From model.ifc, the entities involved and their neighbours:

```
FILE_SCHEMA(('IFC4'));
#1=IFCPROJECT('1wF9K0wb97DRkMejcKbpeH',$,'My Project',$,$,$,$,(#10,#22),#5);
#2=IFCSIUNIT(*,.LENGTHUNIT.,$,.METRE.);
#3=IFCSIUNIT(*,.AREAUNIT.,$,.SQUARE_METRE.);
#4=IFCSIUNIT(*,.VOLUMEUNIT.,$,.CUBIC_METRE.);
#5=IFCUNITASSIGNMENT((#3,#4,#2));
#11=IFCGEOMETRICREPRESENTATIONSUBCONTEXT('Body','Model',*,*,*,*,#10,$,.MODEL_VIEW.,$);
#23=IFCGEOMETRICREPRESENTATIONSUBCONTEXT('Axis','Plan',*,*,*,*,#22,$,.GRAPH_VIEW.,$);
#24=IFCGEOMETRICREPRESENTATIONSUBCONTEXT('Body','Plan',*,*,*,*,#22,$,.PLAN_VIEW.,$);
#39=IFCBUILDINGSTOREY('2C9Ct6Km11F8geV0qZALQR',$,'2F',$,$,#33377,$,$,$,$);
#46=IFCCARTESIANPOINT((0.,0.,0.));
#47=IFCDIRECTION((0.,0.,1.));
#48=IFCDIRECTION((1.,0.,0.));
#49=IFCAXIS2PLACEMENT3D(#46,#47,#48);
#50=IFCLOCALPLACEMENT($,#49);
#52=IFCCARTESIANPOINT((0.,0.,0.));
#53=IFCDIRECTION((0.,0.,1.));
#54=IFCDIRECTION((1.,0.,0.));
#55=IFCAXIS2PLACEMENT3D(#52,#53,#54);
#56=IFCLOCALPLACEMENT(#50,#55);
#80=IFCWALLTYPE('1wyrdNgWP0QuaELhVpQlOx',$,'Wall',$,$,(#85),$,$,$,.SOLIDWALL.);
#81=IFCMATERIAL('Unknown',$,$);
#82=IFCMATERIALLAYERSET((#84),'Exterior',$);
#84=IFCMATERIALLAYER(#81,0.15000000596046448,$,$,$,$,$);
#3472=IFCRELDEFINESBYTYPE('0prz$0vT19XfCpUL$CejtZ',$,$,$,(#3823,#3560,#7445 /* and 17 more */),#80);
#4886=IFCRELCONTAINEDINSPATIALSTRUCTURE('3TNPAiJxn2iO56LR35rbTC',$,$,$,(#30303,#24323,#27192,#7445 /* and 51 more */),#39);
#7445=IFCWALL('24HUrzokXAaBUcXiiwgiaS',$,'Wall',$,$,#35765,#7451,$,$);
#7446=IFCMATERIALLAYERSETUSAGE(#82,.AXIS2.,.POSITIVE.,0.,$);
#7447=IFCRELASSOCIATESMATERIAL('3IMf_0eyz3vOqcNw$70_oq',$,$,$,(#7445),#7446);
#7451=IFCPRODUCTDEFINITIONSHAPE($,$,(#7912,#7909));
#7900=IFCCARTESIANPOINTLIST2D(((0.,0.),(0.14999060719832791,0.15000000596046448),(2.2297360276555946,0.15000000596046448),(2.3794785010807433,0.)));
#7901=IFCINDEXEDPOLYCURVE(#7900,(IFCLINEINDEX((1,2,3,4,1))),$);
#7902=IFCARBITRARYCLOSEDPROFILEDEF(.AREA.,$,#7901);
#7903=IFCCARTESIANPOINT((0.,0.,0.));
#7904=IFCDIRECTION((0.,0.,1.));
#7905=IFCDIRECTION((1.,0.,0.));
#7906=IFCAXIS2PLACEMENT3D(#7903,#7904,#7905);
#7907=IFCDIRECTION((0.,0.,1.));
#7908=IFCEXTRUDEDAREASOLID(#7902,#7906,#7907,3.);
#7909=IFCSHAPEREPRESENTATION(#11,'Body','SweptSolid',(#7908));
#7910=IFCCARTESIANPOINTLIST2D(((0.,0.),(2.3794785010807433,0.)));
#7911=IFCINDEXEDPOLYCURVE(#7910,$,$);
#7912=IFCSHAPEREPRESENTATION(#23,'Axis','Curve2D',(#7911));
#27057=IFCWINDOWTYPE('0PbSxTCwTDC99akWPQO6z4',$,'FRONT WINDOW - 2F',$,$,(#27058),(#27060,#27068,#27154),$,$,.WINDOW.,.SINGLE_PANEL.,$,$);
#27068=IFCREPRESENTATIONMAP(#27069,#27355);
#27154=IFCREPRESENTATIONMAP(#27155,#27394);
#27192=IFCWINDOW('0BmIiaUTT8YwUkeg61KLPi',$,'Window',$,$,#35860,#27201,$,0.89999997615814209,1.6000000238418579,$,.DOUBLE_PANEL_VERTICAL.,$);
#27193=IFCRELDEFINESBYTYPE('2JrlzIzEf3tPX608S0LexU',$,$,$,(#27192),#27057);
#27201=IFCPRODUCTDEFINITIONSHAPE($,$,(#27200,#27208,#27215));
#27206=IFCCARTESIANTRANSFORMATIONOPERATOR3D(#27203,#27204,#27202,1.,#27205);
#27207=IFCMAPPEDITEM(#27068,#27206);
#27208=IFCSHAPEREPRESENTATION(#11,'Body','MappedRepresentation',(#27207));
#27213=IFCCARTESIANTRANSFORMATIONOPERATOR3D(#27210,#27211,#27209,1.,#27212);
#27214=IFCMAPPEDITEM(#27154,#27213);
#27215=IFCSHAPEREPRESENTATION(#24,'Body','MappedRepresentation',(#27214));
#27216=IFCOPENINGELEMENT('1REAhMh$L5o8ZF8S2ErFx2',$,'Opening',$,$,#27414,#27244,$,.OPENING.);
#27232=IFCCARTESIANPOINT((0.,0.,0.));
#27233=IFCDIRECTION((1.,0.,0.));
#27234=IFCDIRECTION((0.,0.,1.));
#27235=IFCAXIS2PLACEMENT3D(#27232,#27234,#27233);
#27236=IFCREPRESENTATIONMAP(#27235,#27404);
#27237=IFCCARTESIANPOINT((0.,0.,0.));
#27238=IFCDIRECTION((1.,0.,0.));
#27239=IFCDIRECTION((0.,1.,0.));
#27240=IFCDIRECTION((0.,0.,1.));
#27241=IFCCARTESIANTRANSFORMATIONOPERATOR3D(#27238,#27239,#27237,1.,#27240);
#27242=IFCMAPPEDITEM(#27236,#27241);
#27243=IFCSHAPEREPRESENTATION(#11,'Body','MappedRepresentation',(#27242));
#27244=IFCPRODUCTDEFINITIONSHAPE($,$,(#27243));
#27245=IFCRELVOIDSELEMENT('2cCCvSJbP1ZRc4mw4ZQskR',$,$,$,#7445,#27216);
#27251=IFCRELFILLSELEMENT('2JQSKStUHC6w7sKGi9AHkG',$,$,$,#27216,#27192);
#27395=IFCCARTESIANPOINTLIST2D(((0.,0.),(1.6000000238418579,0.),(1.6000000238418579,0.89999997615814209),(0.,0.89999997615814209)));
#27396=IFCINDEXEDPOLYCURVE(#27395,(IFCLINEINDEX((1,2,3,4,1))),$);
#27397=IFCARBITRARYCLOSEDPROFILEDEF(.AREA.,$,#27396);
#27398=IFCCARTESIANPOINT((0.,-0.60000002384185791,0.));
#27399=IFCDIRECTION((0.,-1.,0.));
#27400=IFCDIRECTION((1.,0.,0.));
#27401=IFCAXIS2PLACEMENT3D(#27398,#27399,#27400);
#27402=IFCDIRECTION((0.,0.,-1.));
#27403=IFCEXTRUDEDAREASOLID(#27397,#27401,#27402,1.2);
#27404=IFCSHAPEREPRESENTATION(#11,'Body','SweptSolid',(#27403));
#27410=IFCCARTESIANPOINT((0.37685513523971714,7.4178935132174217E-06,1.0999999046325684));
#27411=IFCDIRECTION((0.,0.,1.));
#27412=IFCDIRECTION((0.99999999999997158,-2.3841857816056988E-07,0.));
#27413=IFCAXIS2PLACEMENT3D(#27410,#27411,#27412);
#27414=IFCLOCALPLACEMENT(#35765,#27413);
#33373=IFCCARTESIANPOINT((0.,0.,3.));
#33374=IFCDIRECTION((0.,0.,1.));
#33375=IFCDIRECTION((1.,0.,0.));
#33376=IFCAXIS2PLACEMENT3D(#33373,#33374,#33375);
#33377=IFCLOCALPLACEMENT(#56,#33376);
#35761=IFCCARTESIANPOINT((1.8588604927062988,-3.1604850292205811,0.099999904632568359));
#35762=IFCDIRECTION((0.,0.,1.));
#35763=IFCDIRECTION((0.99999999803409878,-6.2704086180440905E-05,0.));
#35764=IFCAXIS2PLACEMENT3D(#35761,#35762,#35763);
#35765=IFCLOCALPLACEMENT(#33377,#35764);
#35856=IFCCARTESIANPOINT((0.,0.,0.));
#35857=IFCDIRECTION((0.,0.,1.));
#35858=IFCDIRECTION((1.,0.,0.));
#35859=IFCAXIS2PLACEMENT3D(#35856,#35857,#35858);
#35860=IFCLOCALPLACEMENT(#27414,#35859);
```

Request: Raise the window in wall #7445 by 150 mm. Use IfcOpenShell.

```python
import numpy as np
import ifcopenshell
import ifcopenshell.api.geometry
import ifcopenshell.util.placement
import ifcopenshell.util.unit

model = ifcopenshell.open("model.ifc")
unit_scale = ifcopenshell.util.unit.calculate_unit_scale(model)

window = model.by_guid("0BmIiaUTT8YwUkeg61KLPi")
opening = window.FillsVoids[0].RelatingOpeningElement
dz = 0.15

shift = np.array([0.0, 0.0, dz])
# The window is placed relative to its opening, so it follows when the opening moves.
matrix = ifcopenshell.util.placement.get_local_placement(opening.ObjectPlacement)
matrix[:3, 3] += shift
ifcopenshell.api.geometry.edit_object_placement(
    model, product=opening, matrix=matrix, is_si=False, should_transform_children=True
)

print(f"moved by {dz * unit_scale:+.3f} m")

model.write("model_v2.ifc")
```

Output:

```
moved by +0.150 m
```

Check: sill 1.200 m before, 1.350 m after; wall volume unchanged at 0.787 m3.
